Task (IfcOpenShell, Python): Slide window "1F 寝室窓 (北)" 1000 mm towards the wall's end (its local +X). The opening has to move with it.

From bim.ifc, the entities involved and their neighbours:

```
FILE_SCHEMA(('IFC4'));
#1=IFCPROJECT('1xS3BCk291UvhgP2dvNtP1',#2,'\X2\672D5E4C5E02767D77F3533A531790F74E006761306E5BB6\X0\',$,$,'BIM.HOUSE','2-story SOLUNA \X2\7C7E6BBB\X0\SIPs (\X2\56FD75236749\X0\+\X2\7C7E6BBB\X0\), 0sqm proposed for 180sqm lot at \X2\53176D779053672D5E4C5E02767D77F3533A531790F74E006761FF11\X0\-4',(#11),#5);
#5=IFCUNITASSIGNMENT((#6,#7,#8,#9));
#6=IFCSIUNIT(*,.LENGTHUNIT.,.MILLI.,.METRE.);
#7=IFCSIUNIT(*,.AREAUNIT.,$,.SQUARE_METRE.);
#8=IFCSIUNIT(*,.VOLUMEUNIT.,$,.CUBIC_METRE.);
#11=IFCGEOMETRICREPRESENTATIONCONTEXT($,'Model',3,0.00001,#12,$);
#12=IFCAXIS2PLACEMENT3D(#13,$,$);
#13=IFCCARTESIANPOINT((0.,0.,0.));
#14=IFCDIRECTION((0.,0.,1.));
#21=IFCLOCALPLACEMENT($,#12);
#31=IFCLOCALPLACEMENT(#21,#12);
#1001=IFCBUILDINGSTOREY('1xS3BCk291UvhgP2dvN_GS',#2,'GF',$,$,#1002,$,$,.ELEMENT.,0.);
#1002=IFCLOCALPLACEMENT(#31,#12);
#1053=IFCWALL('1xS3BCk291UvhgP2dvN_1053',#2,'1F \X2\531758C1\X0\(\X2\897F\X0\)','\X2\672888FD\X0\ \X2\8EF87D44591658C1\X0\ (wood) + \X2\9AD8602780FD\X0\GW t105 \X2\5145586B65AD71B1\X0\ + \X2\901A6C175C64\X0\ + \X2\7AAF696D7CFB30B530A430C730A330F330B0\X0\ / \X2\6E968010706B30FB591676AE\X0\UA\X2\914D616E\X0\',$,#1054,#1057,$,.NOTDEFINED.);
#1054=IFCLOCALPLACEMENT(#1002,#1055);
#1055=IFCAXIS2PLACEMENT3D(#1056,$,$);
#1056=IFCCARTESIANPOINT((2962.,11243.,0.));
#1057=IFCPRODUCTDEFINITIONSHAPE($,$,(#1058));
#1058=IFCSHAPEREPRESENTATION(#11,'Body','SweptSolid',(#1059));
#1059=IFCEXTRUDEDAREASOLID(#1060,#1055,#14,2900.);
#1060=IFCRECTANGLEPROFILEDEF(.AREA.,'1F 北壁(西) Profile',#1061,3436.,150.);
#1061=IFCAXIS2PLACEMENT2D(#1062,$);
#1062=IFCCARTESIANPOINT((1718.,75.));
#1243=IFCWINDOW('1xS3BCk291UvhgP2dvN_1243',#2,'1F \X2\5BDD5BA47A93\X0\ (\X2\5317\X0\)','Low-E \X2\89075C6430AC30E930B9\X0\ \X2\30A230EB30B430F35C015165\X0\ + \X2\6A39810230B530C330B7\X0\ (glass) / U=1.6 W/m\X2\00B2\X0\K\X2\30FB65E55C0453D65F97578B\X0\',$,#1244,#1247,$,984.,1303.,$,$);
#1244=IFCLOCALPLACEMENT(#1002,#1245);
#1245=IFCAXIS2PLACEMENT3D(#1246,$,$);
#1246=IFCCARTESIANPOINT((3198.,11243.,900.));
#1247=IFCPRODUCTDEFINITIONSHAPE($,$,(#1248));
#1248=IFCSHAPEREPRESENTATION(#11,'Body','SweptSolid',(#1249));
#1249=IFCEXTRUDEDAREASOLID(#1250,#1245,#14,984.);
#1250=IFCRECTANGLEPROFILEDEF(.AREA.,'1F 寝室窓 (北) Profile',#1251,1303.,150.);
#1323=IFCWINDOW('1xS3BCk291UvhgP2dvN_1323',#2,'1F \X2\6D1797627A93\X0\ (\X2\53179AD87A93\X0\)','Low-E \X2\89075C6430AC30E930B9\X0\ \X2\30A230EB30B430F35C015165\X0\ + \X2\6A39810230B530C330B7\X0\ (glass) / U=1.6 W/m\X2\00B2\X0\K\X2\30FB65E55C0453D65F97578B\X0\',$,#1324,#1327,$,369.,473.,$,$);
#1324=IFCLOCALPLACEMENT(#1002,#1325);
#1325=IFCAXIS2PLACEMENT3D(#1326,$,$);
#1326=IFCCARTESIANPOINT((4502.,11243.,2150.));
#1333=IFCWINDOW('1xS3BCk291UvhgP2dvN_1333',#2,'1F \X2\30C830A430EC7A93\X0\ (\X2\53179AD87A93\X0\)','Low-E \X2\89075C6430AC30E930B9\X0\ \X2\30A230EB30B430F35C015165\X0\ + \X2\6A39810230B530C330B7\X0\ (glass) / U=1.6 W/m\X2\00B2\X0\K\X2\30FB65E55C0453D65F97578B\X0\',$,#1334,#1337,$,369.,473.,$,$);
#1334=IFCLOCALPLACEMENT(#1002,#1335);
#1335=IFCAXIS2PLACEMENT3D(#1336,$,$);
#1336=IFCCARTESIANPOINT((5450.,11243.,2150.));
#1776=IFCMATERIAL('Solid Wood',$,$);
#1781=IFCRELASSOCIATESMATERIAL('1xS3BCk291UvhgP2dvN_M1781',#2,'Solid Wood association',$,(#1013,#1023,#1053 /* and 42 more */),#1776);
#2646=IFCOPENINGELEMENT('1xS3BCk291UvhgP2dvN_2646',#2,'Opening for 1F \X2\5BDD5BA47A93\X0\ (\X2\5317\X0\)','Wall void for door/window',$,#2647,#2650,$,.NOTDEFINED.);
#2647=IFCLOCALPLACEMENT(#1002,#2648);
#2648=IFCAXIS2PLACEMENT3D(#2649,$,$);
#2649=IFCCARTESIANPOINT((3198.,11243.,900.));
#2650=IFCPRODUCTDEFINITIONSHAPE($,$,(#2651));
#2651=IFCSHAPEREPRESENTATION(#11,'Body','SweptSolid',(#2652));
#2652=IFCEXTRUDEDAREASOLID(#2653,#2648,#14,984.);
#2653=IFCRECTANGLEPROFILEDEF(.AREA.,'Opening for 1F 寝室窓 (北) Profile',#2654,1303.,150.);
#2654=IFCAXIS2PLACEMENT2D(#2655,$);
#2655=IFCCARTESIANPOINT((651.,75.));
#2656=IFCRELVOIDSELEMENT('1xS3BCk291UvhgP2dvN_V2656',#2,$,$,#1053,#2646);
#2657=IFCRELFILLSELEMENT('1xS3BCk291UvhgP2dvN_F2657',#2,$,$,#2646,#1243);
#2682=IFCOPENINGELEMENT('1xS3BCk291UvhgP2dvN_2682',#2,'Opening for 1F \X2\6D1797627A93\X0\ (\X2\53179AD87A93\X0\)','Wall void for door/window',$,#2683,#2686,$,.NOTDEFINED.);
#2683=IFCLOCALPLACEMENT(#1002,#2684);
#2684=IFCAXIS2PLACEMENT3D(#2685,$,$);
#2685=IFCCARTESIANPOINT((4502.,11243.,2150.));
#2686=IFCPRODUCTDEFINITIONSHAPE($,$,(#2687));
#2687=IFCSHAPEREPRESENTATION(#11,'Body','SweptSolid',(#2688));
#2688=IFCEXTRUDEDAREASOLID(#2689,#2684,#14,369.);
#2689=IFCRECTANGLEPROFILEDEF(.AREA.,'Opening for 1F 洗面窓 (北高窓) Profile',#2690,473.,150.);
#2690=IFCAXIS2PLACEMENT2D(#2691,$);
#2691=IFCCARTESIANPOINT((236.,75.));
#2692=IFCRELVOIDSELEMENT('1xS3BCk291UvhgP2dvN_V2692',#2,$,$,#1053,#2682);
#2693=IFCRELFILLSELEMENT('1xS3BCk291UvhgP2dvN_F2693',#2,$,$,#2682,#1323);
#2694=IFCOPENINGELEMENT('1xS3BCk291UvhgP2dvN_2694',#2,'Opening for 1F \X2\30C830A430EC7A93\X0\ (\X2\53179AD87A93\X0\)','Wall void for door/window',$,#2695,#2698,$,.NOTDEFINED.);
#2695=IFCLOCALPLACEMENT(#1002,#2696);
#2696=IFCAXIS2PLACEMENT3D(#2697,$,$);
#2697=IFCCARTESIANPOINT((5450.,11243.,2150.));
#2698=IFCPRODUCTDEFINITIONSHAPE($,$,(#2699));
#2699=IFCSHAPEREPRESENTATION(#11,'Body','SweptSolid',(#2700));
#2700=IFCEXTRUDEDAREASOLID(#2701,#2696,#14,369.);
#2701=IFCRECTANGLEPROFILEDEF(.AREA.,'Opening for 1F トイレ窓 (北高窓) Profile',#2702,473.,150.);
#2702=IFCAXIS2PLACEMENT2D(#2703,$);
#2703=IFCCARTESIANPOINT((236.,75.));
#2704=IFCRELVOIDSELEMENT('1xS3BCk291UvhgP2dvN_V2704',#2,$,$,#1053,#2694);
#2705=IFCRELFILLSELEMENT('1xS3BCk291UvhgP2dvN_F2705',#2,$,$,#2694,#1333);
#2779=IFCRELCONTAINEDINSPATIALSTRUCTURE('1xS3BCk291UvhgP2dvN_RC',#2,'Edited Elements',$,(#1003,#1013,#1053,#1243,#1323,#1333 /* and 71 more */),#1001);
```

```python
import ifcopenshell
import ifcopenshell.api.geometry
import ifcopenshell.util.placement

model = ifcopenshell.open("bim.ifc")

window = model.by_id(1243)
opening = window.FillsVoids[0].RelatingOpeningElement
wall = opening.VoidsElements[0].RelatingBuildingElement

wall_matrix = ifcopenshell.util.placement.get_local_placement(wall.ObjectPlacement)
shift = wall_matrix[:3, 0] * 1000.0
before = ifcopenshell.util.placement.get_local_placement(window.ObjectPlacement)[:3, 3].copy()

# The window is not placed relative to its opening, so move both.
for product in (opening, window):
    matrix = ifcopenshell.util.placement.get_local_placement(product.ObjectPlacement)
    matrix[:3, 3] += shift
    ifcopenshell.api.geometry.edit_object_placement(model, product=product, matrix=matrix, is_si=False)

after = ifcopenshell.util.placement.get_local_placement(window.ObjectPlacement)[:3, 3]
print("window moved by", (after - before).round(3) + 0.0)

model.write("bim_edited.ifc")
```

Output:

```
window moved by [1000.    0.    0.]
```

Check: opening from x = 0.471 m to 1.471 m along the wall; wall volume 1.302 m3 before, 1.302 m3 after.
